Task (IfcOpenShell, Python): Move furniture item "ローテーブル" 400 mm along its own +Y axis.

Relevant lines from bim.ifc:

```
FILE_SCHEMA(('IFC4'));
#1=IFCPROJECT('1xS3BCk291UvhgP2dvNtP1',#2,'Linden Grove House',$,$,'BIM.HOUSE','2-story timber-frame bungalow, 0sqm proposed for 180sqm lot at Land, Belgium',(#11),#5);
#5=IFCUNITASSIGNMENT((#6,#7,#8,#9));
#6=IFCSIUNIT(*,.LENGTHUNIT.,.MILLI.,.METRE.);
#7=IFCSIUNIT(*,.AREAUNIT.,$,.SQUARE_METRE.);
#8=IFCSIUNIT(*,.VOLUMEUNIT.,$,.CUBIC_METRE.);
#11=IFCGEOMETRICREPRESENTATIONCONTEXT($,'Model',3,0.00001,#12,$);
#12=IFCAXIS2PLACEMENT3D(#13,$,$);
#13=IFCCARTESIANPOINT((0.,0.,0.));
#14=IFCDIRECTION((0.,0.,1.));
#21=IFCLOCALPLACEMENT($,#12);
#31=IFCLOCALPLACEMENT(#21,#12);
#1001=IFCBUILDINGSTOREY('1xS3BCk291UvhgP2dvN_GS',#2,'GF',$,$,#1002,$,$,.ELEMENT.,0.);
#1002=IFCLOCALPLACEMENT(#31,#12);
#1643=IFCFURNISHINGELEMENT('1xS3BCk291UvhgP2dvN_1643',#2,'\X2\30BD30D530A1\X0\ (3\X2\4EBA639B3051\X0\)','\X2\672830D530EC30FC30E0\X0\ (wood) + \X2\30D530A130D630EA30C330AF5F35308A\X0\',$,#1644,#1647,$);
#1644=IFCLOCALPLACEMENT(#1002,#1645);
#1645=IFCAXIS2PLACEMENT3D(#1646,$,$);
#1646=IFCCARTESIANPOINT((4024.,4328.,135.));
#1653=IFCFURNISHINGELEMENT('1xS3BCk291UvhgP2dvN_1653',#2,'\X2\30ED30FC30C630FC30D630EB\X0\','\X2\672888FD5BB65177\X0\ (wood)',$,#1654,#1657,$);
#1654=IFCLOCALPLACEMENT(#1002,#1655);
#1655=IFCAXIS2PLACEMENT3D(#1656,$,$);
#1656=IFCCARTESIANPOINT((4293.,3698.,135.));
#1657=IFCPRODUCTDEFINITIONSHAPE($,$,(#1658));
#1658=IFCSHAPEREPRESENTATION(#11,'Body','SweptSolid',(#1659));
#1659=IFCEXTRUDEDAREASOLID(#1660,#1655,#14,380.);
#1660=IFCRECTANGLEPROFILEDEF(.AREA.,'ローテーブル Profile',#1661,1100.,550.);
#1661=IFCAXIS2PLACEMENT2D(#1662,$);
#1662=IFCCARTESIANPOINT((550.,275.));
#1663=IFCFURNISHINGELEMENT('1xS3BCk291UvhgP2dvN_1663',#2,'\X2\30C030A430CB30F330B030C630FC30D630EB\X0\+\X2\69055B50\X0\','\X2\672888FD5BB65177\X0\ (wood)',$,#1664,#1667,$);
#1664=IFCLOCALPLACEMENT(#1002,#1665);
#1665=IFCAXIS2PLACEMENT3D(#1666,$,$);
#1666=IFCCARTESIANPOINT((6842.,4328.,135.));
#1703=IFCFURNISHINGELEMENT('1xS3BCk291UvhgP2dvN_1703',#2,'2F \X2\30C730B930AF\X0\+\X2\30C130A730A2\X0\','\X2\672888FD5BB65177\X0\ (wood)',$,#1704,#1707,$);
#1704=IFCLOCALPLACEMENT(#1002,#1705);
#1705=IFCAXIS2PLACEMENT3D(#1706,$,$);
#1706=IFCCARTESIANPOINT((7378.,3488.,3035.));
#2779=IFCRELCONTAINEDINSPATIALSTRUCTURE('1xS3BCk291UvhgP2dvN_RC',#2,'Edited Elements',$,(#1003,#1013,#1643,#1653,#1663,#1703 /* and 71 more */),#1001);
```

```python
import ifcopenshell
import ifcopenshell.api.geometry
import ifcopenshell.util.placement
import ifcopenshell.util.unit

model = ifcopenshell.open("bim.ifc")
unit_scale = ifcopenshell.util.unit.calculate_unit_scale(model)

item = model.by_guid("1xS3BCk291UvhgP2dvN_1653")
matrix = ifcopenshell.util.placement.get_local_placement(item.ObjectPlacement)
matrix[:3, 3] += matrix[:3, 1] * 0.4 / unit_scale
ifcopenshell.api.geometry.edit_object_placement(model, product=item, matrix=matrix, is_si=False)

print(ifcopenshell.util.placement.get_local_placement(item.ObjectPlacement).round(3) + 0.0)

model.write("bim_edited.ifc")
```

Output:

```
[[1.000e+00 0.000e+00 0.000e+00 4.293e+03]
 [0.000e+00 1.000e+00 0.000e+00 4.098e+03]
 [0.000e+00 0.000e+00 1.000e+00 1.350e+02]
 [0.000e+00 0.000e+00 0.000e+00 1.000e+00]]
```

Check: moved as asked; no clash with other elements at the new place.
